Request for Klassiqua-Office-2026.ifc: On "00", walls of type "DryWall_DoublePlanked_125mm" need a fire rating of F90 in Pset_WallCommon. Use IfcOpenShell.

First a look at what the model holds.

```python
import ifcopenshell
import ifcopenshell.util.element

model = ifcopenshell.open("Klassiqua-Office-2026.ifc")
print(model.schema)
storey = next(s for s in model.by_type("IfcBuildingStorey") if s.Name == "00")
walls = [e for e in ifcopenshell.util.element.get_decomposition(storey) if e.is_a("IfcWall")]
seen = {}
for e in walls:
    element_type = ifcopenshell.util.element.get_type(e)
    key = (element_type.Name if element_type != e and element_type else None, ifcopenshell.util.element.get_pset(e, "Pset_WallCommon", "FireRating"))
    seen[key] = seen.get(key, 0) + 1
for (name, value), count in sorted(seen.items(), key=str):
    print(count, "x", name, "|", value)
```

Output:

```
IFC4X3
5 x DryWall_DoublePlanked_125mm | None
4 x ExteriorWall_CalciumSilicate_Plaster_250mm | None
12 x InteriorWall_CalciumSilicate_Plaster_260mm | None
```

```python
import ifcopenshell
import ifcopenshell.api.pset
import ifcopenshell.util.element

model = ifcopenshell.open("Klassiqua-Office-2026.ifc")

storey = next(s for s in model.by_type("IfcBuildingStorey") if s.Name == "00")
walls = [e for e in ifcopenshell.util.element.get_decomposition(storey) if e.is_a("IfcWall")]

count = 0
for e in walls:
    element_type = ifcopenshell.util.element.get_type(e)
    if element_type in (None, e) or element_type.Name != "DryWall_DoublePlanked_125mm":
        continue
    # add_pset returns the element's existing set when there is one.
    pset = ifcopenshell.api.pset.add_pset(model, product=e, name="Pset_WallCommon")
    ifcopenshell.api.pset.edit_pset(model, pset=pset, properties={"FireRating": "F90"})
    count += 1

print(count, "walls updated")

model.write("Klassiqua-Office-2026_updated.ifc")
```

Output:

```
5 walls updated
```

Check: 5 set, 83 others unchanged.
